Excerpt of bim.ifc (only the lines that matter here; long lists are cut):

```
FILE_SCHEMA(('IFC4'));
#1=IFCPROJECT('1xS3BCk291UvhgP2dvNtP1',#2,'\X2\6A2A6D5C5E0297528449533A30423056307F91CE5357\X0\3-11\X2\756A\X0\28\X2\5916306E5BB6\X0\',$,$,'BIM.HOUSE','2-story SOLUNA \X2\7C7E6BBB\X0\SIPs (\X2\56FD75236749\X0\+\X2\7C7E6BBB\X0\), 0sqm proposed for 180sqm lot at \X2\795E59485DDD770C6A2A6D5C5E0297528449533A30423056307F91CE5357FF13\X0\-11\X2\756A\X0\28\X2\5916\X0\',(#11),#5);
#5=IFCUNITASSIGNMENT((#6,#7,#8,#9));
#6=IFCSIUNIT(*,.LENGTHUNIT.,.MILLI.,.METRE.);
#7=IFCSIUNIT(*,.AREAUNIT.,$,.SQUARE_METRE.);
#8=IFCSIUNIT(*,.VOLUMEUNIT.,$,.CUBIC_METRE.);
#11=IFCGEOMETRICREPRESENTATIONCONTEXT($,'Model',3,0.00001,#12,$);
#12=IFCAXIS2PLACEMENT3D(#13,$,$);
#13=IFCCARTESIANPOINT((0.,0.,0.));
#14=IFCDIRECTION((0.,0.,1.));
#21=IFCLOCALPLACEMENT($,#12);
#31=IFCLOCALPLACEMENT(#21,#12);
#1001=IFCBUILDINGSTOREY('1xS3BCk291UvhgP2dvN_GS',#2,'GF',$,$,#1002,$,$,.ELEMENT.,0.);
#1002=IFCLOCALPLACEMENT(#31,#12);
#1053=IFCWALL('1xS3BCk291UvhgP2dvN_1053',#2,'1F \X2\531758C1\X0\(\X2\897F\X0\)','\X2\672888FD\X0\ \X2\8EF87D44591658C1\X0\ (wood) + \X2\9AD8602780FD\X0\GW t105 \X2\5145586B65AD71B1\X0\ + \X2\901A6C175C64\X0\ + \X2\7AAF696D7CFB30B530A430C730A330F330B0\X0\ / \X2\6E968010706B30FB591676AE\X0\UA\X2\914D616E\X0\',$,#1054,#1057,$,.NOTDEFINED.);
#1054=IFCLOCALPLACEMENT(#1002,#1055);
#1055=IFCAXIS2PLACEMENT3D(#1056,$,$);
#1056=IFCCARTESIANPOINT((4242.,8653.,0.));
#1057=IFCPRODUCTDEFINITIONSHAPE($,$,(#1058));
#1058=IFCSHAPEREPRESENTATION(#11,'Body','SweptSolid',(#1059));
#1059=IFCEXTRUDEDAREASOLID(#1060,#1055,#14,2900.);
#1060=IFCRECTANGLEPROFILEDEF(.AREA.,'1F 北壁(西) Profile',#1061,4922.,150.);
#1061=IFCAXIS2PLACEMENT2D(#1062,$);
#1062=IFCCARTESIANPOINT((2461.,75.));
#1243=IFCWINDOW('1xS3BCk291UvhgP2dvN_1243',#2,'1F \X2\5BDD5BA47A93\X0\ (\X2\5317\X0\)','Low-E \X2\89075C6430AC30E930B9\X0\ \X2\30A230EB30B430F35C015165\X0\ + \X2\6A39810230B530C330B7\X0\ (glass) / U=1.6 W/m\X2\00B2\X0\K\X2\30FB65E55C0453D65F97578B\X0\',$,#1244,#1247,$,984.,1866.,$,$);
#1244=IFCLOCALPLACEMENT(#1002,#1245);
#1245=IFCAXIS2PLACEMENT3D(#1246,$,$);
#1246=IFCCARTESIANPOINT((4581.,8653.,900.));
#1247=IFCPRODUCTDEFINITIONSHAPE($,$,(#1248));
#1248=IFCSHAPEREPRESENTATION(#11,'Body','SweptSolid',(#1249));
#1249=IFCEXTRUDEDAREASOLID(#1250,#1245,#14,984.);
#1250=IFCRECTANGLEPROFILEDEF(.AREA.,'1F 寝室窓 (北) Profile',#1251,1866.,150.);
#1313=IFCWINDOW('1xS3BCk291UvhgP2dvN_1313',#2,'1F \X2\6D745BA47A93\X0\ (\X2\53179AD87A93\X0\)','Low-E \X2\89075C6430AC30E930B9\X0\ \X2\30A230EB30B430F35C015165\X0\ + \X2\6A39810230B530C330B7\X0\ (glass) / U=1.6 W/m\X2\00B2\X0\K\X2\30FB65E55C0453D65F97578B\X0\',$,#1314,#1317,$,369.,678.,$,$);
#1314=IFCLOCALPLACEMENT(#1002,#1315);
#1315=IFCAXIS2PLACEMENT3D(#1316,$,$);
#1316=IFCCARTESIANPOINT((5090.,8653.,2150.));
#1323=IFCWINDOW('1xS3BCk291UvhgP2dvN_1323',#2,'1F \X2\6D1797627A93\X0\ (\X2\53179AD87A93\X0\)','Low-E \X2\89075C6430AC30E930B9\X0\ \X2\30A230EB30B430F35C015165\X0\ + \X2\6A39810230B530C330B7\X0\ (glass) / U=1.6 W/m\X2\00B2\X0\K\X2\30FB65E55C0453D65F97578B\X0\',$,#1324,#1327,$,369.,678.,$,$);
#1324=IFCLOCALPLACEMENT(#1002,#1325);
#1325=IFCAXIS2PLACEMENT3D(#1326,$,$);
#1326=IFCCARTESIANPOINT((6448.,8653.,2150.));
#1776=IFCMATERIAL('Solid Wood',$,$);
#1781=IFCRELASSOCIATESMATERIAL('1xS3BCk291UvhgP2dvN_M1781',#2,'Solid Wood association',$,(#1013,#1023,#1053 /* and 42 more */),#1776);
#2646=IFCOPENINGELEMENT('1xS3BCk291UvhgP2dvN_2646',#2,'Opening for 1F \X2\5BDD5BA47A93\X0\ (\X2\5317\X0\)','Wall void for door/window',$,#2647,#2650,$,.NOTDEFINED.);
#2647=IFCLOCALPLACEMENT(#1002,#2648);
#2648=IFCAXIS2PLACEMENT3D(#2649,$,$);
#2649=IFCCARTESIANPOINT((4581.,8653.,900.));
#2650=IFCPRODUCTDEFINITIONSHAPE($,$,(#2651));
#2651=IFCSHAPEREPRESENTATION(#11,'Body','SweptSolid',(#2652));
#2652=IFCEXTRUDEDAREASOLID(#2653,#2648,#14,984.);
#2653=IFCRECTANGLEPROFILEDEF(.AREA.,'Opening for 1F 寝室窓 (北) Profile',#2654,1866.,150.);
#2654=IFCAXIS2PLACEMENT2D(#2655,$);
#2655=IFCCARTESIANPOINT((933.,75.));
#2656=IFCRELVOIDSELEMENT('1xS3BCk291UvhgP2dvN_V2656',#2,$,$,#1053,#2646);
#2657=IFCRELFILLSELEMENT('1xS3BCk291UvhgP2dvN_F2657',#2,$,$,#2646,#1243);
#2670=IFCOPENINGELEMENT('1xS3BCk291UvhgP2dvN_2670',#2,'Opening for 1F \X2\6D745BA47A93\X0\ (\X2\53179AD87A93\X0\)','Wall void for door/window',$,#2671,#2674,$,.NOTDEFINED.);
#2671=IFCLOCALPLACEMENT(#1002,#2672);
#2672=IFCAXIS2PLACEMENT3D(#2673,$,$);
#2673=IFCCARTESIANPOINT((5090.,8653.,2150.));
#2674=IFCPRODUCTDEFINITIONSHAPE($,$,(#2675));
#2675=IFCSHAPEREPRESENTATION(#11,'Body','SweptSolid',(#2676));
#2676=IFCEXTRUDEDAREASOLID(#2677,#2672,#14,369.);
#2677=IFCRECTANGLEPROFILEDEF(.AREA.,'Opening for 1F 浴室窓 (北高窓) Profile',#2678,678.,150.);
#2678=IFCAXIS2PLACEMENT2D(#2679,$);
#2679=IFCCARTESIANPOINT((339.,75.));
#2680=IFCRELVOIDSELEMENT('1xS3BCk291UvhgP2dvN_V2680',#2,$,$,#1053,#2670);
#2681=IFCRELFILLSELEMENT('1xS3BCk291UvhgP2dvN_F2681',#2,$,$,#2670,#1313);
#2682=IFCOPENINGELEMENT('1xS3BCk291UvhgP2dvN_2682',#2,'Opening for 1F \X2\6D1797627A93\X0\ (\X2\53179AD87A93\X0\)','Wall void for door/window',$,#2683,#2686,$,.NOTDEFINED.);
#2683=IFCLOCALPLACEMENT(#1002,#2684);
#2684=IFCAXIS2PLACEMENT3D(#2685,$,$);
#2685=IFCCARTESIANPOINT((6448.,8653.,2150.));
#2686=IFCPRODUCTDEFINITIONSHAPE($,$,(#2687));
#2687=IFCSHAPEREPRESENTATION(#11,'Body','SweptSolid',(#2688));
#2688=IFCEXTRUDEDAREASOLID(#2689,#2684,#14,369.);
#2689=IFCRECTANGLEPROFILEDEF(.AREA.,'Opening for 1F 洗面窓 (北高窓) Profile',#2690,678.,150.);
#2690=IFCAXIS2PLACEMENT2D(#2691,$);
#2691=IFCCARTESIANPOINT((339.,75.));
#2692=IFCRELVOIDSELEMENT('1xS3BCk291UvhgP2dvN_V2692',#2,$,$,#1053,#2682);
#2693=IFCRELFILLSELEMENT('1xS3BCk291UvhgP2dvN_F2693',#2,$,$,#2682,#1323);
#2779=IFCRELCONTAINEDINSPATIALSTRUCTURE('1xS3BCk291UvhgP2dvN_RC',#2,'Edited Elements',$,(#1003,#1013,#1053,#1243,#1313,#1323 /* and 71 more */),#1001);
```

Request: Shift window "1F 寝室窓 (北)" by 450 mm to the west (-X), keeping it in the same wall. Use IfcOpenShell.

```python
import ifcopenshell
import ifcopenshell.api.geometry
import ifcopenshell.util.placement
import ifcopenshell.util.unit

model = ifcopenshell.open("bim.ifc")
unit_scale = ifcopenshell.util.unit.calculate_unit_scale(model)

window = model.by_guid("1xS3BCk291UvhgP2dvN_1243")
opening = window.FillsVoids[0].RelatingOpeningElement
wall = opening.VoidsElements[0].RelatingBuildingElement

wall_matrix = ifcopenshell.util.placement.get_local_placement(wall.ObjectPlacement)
shift = wall_matrix[:3, 0] * -0.45 / unit_scale
before = ifcopenshell.util.placement.get_local_placement(window.ObjectPlacement)[:3, 3].copy()

# The window is not placed relative to its opening, so move both.
for product in (opening, window):
    matrix = ifcopenshell.util.placement.get_local_placement(product.ObjectPlacement)
    matrix[:3, 3] += shift
    ifcopenshell.api.geometry.edit_object_placement(model, product=product, matrix=matrix, is_si=False)

after = ifcopenshell.util.placement.get_local_placement(window.ObjectPlacement)[:3, 3]
print("window moved by", (after - before).round(3) + 0.0)

model.write("bim_edited.ifc")
```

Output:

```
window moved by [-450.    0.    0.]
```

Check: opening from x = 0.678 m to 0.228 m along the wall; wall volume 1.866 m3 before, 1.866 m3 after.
